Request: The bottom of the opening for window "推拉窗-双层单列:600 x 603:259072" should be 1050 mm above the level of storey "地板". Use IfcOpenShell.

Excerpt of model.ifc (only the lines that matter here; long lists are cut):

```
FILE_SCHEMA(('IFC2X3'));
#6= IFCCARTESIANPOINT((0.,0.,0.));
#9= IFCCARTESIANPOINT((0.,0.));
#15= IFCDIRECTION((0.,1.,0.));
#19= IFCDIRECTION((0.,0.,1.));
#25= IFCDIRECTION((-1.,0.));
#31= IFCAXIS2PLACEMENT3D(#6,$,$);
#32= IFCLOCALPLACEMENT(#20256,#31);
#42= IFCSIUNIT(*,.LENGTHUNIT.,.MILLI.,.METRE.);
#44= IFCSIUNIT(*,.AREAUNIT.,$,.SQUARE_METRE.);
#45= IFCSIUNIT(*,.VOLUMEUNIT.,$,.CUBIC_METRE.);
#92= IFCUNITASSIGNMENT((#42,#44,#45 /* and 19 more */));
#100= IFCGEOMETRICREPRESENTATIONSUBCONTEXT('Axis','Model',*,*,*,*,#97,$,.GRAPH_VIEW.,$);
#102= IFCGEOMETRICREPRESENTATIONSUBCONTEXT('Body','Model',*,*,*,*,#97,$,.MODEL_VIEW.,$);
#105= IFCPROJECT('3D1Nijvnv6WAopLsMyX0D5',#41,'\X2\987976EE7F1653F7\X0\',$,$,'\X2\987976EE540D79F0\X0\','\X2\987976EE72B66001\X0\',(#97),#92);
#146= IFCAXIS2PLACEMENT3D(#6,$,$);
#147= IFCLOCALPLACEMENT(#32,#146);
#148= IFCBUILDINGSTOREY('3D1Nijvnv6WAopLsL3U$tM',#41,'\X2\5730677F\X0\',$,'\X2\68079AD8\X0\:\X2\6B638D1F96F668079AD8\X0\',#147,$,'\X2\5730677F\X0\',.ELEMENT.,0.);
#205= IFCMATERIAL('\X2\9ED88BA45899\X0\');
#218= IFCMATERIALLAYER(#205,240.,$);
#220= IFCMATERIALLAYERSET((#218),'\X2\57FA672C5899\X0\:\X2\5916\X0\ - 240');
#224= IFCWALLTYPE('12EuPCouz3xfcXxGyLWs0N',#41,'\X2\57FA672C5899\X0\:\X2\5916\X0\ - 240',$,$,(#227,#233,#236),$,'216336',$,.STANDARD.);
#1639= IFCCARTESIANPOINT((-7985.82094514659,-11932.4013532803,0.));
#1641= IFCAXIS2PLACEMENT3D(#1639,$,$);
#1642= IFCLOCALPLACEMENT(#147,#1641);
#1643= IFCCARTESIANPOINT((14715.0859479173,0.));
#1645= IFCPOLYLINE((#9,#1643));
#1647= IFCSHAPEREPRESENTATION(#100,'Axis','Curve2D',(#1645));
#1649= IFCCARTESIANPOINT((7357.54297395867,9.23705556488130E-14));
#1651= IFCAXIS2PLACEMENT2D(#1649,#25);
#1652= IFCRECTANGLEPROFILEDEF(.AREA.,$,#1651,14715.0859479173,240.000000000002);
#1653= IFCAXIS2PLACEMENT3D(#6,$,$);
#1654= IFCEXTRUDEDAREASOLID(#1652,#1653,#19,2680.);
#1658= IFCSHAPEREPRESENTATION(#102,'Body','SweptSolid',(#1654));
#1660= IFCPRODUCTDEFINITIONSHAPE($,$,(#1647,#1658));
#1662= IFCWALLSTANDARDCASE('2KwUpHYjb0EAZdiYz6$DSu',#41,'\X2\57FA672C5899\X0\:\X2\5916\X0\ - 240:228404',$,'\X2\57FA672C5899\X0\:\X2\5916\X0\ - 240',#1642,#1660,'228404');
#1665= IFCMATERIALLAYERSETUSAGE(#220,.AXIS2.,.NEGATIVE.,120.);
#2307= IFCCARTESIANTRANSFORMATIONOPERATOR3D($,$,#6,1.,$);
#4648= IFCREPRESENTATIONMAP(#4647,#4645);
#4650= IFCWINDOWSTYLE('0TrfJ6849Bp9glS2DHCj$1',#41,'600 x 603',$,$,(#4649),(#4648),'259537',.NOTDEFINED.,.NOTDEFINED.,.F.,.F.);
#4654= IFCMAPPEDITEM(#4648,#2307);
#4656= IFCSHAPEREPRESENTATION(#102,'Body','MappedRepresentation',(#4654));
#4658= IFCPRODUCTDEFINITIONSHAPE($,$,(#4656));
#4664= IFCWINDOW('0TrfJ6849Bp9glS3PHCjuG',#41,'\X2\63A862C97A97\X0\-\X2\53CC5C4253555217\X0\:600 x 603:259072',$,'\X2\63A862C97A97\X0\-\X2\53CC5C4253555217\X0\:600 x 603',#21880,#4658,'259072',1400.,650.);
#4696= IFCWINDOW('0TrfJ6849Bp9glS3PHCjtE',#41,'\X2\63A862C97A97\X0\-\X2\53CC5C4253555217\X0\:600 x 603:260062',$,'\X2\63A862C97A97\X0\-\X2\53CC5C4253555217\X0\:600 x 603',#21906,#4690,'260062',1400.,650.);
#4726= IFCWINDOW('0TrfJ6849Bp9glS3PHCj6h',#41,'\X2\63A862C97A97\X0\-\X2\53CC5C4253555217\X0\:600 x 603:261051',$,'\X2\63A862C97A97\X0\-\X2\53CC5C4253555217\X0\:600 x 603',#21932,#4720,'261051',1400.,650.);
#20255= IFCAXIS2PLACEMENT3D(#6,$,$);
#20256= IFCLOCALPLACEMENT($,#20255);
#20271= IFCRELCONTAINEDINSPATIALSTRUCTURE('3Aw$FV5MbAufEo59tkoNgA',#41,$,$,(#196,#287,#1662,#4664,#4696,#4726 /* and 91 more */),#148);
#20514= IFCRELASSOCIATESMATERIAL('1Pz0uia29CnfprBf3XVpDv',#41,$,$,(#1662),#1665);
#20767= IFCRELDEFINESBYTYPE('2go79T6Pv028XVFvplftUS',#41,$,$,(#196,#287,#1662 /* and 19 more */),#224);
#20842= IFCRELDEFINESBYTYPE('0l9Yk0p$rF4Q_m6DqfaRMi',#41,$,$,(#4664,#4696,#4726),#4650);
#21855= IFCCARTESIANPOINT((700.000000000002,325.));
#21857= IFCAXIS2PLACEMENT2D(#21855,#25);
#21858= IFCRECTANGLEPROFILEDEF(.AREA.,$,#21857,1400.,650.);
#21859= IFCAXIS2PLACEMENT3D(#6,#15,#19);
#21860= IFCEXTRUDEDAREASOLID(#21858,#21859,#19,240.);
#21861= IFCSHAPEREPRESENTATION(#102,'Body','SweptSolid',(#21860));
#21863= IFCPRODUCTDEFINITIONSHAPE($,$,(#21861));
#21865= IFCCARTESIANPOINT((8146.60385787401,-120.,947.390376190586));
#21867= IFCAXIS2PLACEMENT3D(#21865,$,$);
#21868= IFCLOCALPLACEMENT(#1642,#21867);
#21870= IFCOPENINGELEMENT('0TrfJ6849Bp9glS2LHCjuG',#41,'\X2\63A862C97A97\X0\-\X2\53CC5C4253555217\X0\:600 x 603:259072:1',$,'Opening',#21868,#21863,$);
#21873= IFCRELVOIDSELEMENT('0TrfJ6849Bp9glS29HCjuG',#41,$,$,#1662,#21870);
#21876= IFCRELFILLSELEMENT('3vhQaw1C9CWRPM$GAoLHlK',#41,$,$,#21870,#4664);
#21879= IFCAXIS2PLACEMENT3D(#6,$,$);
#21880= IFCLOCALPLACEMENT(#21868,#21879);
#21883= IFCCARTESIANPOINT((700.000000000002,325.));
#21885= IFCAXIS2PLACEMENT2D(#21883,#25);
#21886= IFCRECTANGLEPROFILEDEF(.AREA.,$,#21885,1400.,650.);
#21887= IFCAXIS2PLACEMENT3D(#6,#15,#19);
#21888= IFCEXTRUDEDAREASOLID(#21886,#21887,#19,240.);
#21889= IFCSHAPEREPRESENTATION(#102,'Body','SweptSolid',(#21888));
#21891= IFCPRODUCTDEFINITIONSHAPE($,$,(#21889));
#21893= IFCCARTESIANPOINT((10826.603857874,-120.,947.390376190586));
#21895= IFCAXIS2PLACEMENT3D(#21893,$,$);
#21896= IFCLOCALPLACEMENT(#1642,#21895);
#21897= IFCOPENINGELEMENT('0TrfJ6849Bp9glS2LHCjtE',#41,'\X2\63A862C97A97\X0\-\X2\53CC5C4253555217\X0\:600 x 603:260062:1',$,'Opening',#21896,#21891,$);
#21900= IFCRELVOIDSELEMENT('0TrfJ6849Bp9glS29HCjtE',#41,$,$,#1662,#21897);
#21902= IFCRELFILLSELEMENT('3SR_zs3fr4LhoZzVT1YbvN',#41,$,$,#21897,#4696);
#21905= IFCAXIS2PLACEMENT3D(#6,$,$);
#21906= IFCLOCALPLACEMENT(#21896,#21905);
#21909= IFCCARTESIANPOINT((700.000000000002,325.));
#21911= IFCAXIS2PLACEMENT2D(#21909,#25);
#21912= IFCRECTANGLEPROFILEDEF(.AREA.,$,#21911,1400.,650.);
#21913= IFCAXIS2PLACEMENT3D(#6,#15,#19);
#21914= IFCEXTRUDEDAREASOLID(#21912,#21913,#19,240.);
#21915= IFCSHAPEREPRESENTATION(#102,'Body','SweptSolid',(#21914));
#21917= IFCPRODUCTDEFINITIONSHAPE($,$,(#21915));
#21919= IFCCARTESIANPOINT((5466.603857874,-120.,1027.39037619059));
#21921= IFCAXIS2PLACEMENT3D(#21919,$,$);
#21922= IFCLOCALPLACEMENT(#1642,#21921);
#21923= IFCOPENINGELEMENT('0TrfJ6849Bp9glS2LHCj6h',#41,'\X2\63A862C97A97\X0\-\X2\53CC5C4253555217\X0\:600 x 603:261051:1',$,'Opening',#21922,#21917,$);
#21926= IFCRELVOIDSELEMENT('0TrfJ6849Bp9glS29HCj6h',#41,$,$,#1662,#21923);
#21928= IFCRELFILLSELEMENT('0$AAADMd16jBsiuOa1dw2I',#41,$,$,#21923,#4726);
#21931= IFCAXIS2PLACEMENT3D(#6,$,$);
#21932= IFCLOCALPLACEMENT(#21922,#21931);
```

```python
import numpy as np
import ifcopenshell
import ifcopenshell.api.geometry
import ifcopenshell.geom
import ifcopenshell.util.element
import ifcopenshell.util.placement
import ifcopenshell.util.shape
import ifcopenshell.util.unit

model = ifcopenshell.open("model.ifc")
unit_scale = ifcopenshell.util.unit.calculate_unit_scale(model)

window = model.by_guid("0TrfJ6849Bp9glS3PHCjuG")
opening = window.FillsVoids[0].RelatingOpeningElement
storey = ifcopenshell.util.element.get_container(window, ifc_class="IfcBuildingStorey")
level = ifcopenshell.util.placement.get_local_placement(storey.ObjectPlacement)[2, 3]

# The opening's origin need not be at the sill, so measure its lowest point.
shape = ifcopenshell.geom.create_shape(ifcopenshell.geom.settings(), opening)
bottom = ifcopenshell.util.shape.get_shape_bottom_elevation(shape, shape.geometry) / unit_scale
dz = level + 1050.0 - bottom

shift = np.array([0.0, 0.0, dz])
# The window is placed relative to its opening, so it follows when the opening moves.
matrix = ifcopenshell.util.placement.get_local_placement(opening.ObjectPlacement)
matrix[:3, 3] += shift
ifcopenshell.api.geometry.edit_object_placement(
    model, product=opening, matrix=matrix, is_si=False, should_transform_children=True
)

print(f"moved by {dz * unit_scale:+.3f} m")

model.write("model_updated.ifc")
```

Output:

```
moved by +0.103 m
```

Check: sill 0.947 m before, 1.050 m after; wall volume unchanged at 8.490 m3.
